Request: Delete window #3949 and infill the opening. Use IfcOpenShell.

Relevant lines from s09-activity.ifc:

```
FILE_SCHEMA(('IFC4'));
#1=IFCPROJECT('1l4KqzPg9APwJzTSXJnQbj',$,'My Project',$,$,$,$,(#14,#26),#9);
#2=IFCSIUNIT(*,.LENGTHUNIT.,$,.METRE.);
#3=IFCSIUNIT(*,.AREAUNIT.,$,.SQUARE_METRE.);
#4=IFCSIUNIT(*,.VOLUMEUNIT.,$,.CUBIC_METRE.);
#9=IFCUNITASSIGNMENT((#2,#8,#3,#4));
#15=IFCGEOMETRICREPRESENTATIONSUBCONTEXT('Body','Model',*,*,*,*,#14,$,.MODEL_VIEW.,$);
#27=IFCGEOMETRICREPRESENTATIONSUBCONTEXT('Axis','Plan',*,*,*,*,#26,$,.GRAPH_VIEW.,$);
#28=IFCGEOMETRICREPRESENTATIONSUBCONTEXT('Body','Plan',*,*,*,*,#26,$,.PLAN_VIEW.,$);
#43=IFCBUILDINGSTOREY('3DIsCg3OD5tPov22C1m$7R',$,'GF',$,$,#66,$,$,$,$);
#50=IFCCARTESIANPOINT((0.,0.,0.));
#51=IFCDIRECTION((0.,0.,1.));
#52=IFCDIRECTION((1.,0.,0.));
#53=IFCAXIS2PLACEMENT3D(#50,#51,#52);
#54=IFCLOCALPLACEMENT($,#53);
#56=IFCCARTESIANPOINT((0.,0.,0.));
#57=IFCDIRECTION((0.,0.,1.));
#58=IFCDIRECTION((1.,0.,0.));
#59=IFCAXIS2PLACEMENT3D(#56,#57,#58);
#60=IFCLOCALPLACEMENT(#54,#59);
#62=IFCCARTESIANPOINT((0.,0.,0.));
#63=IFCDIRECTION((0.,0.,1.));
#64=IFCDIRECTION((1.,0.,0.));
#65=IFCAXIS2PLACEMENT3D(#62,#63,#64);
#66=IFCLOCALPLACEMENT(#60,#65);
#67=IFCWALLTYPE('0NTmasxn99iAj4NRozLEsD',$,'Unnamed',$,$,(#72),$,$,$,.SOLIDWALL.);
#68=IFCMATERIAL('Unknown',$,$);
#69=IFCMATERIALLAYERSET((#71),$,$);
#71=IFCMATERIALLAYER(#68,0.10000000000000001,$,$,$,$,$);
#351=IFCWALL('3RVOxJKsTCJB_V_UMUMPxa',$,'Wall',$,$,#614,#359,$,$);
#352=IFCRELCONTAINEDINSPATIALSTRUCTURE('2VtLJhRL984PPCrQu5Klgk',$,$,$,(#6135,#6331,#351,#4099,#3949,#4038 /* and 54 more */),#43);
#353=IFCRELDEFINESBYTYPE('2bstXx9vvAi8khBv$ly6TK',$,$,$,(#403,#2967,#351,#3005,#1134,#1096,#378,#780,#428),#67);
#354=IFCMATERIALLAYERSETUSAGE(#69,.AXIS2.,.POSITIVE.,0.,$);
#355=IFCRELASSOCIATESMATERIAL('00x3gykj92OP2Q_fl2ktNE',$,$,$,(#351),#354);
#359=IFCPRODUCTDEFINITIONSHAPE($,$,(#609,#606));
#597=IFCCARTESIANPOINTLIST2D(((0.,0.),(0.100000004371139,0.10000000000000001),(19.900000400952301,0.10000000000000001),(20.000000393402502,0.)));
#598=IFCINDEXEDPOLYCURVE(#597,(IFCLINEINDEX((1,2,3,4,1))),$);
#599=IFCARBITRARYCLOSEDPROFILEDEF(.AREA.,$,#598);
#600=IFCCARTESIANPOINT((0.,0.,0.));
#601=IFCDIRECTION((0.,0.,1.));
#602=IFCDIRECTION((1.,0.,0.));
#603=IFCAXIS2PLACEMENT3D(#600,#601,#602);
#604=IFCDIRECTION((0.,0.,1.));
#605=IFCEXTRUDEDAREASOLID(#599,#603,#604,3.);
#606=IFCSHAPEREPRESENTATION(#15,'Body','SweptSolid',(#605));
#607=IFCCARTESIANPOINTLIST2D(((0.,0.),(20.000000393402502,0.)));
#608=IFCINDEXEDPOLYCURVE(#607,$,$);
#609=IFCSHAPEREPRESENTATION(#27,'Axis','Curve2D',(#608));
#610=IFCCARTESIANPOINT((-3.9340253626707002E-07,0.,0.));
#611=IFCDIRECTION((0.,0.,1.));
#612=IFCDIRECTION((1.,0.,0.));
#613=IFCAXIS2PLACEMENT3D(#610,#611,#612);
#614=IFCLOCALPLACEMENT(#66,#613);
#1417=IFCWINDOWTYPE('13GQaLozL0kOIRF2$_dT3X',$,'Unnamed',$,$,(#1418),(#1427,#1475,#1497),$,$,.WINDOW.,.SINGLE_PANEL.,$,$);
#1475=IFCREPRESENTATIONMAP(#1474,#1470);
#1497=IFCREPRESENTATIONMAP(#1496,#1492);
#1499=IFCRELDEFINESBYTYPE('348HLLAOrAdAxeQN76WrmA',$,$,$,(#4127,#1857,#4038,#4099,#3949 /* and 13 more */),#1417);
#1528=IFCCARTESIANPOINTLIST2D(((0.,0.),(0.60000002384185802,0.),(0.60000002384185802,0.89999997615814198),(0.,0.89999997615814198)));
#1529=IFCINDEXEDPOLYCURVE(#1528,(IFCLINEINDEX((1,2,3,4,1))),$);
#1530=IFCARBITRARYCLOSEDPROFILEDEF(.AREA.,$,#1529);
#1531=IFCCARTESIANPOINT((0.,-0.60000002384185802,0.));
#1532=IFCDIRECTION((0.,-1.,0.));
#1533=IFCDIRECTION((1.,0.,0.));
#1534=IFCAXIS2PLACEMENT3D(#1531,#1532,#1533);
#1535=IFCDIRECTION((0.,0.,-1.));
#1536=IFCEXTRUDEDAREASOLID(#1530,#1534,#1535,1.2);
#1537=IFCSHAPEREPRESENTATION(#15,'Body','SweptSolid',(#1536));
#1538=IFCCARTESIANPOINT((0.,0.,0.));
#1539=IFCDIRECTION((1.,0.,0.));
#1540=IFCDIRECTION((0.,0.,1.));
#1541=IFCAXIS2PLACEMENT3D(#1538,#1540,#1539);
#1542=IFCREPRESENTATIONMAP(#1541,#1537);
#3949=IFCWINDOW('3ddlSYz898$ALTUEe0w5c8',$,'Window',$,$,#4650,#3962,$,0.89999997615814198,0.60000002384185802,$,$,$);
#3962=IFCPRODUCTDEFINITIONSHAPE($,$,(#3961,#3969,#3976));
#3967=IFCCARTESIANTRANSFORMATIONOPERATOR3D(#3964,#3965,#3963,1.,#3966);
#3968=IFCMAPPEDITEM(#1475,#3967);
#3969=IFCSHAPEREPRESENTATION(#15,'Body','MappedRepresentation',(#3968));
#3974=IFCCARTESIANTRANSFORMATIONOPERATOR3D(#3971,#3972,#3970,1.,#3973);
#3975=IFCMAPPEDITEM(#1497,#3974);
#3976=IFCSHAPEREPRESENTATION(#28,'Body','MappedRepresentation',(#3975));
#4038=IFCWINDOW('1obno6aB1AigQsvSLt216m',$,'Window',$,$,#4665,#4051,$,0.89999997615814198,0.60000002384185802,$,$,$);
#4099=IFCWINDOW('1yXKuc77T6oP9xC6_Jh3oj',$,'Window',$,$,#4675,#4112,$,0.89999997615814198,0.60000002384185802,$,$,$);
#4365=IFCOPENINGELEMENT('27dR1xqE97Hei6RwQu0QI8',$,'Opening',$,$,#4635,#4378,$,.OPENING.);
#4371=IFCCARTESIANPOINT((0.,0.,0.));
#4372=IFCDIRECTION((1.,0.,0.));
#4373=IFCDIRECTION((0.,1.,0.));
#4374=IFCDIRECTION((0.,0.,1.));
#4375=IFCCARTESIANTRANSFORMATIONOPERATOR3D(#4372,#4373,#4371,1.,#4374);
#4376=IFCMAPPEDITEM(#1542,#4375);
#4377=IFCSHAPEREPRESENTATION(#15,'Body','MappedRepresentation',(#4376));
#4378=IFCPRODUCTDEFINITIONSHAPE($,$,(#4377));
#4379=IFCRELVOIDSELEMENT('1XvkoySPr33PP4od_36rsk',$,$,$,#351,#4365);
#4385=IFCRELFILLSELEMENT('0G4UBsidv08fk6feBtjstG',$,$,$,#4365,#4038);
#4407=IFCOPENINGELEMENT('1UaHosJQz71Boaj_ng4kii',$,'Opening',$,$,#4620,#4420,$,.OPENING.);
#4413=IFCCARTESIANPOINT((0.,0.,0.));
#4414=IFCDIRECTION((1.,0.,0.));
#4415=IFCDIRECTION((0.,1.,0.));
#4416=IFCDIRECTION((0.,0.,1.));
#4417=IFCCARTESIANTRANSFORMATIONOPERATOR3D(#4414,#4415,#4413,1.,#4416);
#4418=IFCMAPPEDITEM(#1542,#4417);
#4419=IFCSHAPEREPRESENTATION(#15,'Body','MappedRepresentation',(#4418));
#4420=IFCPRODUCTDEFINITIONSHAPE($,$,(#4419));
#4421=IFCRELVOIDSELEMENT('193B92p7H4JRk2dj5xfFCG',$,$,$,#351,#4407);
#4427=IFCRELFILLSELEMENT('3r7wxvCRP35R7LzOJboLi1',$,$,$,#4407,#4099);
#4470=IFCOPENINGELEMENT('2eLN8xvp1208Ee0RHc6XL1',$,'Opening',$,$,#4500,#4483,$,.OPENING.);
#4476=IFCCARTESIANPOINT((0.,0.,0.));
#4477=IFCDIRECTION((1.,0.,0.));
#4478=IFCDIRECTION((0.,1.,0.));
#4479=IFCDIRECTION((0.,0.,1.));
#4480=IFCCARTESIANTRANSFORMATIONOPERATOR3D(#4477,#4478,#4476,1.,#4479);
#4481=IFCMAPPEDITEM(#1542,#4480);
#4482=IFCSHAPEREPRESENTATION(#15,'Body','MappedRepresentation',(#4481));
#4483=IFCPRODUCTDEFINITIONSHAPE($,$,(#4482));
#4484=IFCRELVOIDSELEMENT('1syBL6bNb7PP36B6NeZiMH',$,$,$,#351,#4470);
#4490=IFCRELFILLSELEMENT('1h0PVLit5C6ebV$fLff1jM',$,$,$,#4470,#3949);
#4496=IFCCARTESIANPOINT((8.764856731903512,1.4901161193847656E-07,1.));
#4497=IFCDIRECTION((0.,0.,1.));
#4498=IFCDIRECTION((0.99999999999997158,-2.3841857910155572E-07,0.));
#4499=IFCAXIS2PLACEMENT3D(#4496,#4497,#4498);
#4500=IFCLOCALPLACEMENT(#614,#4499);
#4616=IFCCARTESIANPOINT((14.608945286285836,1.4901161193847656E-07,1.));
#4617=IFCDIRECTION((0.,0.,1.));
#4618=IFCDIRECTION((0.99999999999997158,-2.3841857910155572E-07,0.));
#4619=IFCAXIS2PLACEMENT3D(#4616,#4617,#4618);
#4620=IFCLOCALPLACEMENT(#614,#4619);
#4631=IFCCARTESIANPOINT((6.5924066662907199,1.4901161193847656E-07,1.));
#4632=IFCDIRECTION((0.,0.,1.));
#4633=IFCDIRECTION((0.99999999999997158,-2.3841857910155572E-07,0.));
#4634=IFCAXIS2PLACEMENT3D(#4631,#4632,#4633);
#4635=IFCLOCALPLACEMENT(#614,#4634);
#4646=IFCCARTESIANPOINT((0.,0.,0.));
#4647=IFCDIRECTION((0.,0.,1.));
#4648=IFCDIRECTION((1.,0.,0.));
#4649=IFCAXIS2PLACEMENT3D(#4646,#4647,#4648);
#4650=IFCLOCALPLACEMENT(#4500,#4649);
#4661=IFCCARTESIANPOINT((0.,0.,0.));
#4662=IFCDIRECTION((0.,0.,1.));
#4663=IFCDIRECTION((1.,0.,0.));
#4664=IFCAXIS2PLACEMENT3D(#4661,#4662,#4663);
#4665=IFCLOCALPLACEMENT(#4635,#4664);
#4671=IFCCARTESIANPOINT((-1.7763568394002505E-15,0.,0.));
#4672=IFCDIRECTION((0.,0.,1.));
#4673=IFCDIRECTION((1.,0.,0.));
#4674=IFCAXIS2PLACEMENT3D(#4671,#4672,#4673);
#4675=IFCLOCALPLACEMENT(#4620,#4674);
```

```python
import ifcopenshell
import ifcopenshell.api.feature
import ifcopenshell.api.root
import ifcopenshell.geom
import ifcopenshell.util.shape

model = ifcopenshell.open("s09-activity.ifc")
settings = ifcopenshell.geom.settings()


def volume(element):
    """Net volume in cubic metres, openings subtracted."""
    shape = ifcopenshell.geom.create_shape(settings, element)
    return ifcopenshell.util.shape.get_volume(shape.geometry)


window = model.by_guid("3ddlSYz898$ALTUEe0w5c8")
opening = window.FillsVoids[0].RelatingOpeningElement
wall = opening.VoidsElements[0].RelatingBuildingElement
before = volume(wall)

ifcopenshell.api.root.remove_product(model, product=window)
ifcopenshell.api.feature.remove_feature(model, feature=opening)

after = volume(wall)

print(f"wall volume {before:.3f} -> {after:.3f} m3")

model.write("s09-activity_rev.ifc")
```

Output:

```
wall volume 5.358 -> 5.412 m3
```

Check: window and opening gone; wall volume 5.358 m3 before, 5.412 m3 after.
